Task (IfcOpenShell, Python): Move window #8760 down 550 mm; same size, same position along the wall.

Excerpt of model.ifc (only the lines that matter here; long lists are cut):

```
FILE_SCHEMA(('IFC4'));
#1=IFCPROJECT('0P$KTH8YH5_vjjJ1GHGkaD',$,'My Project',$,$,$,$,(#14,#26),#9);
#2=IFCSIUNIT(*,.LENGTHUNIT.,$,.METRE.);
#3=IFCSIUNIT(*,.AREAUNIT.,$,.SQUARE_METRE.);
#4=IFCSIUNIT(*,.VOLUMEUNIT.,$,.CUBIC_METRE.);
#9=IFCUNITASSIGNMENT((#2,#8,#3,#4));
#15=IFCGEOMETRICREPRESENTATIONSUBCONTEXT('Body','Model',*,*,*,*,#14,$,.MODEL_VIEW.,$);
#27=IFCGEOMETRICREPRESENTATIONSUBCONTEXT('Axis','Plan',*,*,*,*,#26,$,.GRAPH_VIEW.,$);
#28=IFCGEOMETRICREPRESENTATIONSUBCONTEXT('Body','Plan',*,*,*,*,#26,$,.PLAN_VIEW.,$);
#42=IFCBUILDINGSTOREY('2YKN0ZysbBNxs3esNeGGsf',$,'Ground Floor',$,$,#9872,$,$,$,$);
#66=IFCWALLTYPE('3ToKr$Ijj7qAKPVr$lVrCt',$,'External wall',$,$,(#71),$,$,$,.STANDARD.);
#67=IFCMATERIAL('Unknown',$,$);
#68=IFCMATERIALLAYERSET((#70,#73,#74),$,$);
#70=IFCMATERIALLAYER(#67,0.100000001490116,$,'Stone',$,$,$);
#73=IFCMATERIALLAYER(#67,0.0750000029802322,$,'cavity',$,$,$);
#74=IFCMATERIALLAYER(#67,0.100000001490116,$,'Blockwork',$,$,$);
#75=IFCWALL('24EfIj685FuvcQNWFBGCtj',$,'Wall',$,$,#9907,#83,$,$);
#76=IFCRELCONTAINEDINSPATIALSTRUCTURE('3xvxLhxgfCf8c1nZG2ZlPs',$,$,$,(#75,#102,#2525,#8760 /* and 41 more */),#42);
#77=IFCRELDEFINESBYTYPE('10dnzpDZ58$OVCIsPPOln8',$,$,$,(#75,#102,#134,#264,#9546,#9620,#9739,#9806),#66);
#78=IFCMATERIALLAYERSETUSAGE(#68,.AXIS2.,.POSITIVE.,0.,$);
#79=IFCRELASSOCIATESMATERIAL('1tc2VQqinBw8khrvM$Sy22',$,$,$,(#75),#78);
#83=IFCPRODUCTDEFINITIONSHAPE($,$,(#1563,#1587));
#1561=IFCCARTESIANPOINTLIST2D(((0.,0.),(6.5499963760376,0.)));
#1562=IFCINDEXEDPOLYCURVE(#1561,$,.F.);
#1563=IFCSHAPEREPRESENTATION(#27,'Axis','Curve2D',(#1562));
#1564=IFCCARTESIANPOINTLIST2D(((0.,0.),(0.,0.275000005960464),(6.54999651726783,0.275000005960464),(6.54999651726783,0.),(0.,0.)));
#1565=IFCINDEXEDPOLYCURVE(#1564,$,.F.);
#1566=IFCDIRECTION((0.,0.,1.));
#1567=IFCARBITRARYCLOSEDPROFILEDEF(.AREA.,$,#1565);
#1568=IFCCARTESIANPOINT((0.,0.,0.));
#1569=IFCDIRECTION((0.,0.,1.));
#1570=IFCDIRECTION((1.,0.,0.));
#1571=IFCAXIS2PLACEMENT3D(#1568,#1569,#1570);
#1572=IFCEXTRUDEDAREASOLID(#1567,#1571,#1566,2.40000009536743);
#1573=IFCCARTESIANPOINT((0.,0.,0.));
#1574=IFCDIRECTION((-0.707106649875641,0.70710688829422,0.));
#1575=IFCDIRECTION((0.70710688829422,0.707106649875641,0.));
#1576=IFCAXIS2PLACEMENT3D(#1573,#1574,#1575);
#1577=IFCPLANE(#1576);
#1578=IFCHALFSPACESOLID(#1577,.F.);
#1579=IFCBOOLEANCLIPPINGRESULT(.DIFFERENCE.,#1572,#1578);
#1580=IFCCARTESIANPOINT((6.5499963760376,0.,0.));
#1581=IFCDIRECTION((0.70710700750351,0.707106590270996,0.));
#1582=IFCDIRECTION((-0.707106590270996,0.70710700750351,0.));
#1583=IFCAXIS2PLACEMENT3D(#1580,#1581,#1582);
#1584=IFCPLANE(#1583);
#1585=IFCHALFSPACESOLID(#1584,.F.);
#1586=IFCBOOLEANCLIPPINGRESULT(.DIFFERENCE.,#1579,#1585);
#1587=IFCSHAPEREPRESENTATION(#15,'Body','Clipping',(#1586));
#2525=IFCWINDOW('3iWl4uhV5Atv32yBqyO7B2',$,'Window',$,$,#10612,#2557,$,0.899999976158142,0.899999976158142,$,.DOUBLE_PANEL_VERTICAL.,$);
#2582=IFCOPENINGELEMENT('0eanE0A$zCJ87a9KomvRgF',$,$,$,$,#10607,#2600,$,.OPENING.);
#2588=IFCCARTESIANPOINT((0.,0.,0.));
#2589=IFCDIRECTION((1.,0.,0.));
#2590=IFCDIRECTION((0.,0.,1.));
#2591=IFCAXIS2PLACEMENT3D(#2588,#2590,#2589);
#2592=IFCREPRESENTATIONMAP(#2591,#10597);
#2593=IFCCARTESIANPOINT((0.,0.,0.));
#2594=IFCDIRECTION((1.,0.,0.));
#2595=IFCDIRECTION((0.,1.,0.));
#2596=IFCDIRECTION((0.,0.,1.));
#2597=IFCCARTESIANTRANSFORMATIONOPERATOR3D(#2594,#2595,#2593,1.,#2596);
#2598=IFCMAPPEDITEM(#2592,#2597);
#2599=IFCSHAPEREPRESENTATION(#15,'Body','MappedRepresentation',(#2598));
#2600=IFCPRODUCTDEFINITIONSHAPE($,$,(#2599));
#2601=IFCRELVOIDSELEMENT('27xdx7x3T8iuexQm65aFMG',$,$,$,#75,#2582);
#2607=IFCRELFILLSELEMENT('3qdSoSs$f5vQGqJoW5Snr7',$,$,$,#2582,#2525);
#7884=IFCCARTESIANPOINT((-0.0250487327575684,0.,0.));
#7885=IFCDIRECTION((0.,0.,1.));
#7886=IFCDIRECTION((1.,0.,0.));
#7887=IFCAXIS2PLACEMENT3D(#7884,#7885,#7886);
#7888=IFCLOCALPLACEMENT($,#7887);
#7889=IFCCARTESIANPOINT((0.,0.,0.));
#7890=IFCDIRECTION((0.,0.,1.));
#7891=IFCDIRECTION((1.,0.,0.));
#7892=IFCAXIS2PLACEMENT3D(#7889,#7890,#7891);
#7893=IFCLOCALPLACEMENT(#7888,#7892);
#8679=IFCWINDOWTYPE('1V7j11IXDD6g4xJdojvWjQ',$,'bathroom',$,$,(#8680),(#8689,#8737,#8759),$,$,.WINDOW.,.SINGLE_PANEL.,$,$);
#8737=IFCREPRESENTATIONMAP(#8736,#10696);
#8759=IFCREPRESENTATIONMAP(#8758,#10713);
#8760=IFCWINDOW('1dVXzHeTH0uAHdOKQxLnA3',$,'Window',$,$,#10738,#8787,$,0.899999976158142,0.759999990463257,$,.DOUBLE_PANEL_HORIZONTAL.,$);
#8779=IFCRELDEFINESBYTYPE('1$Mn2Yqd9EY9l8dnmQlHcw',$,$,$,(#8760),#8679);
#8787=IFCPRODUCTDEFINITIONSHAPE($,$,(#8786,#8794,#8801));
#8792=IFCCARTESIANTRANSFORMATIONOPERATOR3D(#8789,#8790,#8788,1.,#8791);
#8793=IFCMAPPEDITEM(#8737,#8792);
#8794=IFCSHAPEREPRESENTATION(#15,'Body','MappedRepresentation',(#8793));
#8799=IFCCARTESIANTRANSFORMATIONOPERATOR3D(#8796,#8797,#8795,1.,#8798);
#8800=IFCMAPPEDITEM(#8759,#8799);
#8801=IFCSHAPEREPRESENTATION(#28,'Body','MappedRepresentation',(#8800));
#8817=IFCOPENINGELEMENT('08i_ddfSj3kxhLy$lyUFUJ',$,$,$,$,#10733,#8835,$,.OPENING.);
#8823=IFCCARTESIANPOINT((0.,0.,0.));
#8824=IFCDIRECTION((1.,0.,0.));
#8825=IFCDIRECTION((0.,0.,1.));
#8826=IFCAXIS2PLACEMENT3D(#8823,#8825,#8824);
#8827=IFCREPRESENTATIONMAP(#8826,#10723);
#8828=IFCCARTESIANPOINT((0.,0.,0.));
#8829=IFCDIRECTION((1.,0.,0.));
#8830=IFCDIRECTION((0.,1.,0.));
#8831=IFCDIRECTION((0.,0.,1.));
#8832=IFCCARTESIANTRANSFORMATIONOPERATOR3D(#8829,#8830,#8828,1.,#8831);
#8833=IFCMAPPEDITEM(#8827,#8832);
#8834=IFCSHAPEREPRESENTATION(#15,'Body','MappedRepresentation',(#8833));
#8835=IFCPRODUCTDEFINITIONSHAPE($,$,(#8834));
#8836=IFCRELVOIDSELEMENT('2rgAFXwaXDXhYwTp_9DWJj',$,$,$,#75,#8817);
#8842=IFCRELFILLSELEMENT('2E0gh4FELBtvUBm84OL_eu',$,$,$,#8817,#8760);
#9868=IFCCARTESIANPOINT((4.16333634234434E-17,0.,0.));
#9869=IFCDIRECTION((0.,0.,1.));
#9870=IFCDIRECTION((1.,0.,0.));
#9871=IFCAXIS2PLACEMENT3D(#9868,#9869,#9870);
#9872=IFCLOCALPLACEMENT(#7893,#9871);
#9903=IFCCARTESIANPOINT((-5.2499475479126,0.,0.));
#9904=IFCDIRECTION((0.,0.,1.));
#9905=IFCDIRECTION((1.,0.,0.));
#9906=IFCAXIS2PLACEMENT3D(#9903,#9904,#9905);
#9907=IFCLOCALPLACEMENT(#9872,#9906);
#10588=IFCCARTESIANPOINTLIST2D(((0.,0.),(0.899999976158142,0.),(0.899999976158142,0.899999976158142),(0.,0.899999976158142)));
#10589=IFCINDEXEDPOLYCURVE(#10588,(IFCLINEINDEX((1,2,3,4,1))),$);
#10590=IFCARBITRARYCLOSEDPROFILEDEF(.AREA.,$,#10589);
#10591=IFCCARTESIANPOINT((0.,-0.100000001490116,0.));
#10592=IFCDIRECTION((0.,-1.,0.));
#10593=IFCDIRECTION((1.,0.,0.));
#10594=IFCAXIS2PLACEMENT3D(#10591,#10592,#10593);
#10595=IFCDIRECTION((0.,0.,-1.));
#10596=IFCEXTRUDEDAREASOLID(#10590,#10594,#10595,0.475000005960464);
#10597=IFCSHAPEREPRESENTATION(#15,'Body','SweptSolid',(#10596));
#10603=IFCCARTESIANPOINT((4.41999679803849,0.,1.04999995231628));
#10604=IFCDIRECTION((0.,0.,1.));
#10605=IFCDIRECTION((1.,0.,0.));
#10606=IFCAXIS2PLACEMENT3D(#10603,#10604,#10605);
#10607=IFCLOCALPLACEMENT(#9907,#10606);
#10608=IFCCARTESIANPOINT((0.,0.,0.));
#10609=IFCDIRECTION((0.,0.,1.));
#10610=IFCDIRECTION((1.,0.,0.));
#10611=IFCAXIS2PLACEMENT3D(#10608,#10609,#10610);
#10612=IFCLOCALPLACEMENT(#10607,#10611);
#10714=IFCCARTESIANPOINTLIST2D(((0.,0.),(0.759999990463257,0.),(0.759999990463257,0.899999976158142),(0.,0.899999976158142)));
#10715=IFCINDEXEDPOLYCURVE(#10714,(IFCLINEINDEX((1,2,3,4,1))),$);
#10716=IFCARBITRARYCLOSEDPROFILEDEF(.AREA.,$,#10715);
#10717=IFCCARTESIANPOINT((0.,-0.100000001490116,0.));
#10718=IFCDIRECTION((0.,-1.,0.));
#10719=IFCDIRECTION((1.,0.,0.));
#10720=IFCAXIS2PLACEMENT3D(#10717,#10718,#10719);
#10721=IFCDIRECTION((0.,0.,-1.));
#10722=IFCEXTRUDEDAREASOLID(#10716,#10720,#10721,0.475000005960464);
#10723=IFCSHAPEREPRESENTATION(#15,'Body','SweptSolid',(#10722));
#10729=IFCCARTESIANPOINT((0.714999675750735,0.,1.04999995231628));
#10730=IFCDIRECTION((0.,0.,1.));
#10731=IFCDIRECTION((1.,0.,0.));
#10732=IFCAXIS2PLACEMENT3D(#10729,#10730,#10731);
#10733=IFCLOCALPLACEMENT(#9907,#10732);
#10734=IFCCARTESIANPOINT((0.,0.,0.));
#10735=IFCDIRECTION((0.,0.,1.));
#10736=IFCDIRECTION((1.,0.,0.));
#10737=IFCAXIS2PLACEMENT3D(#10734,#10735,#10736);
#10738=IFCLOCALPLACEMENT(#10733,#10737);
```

```python
import numpy as np
import ifcopenshell
import ifcopenshell.api.geometry
import ifcopenshell.util.placement
import ifcopenshell.util.unit

model = ifcopenshell.open("model.ifc")
unit_scale = ifcopenshell.util.unit.calculate_unit_scale(model)

window = model.by_guid("1dVXzHeTH0uAHdOKQxLnA3")
opening = window.FillsVoids[0].RelatingOpeningElement
dz = -0.55

shift = np.array([0.0, 0.0, dz])
# The window is placed relative to its opening, so it follows when the opening moves.
matrix = ifcopenshell.util.placement.get_local_placement(opening.ObjectPlacement)
matrix[:3, 3] += shift
ifcopenshell.api.geometry.edit_object_placement(
    model, product=opening, matrix=matrix, is_si=False, should_transform_children=True
)

print(f"moved by {dz * unit_scale:+.3f} m")

model.write("model_updated.ifc")
```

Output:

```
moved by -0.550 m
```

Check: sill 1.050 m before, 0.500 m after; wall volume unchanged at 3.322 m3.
